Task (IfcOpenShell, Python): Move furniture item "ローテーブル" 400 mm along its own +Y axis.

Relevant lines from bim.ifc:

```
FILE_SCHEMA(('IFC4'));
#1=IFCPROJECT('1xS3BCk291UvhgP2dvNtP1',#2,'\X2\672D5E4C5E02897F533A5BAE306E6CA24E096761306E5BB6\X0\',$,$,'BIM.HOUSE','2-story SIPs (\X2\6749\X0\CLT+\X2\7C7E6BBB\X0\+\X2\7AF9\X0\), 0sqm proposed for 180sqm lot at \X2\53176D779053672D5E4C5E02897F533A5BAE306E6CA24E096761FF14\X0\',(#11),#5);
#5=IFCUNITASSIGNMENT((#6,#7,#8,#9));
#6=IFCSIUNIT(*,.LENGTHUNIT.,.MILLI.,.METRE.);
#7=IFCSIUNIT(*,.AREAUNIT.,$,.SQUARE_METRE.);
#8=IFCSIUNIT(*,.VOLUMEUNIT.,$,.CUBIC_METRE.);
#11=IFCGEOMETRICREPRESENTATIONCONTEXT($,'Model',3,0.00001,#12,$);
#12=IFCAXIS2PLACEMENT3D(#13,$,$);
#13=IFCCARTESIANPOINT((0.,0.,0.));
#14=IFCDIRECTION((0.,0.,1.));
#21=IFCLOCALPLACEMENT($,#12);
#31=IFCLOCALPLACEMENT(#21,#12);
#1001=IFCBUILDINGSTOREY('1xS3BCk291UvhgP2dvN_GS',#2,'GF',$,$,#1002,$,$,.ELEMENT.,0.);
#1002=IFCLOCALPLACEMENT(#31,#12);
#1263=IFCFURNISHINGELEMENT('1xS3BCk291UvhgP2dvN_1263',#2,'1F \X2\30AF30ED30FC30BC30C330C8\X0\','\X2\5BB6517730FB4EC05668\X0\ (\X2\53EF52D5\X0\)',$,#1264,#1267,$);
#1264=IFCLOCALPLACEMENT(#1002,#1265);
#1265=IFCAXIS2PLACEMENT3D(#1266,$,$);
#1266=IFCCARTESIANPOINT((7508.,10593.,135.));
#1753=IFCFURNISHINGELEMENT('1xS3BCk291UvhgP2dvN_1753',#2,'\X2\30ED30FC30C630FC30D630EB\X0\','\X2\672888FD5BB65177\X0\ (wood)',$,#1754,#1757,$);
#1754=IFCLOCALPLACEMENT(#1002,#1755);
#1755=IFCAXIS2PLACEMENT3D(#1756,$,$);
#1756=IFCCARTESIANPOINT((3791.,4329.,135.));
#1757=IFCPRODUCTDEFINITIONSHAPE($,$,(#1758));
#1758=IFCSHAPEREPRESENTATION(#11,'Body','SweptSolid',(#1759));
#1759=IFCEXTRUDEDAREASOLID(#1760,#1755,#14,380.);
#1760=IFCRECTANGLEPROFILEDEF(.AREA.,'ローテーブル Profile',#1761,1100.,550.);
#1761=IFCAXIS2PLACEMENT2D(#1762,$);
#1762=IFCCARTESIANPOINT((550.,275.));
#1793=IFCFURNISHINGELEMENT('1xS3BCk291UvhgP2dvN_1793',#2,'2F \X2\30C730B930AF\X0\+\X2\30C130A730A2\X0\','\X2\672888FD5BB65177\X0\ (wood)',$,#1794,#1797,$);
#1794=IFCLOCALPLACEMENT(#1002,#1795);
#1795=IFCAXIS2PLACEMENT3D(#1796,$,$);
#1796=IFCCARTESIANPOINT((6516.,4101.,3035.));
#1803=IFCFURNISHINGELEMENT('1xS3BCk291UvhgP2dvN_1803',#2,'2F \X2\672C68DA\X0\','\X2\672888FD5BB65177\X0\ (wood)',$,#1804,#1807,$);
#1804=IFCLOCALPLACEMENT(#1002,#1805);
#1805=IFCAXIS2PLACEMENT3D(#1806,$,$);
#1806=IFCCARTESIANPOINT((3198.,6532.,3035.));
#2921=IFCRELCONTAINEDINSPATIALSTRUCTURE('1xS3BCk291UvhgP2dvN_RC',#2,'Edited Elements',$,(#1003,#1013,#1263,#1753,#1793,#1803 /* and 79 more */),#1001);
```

```python
import ifcopenshell
import ifcopenshell.api.geometry
import ifcopenshell.util.placement
import ifcopenshell.util.unit

model = ifcopenshell.open("bim.ifc")
unit_scale = ifcopenshell.util.unit.calculate_unit_scale(model)

item = model.by_id(1753)
matrix = ifcopenshell.util.placement.get_local_placement(item.ObjectPlacement)
matrix[:3, 3] += matrix[:3, 1] * 0.4 / unit_scale
ifcopenshell.api.geometry.edit_object_placement(model, product=item, matrix=matrix, is_si=False)

print(ifcopenshell.util.placement.get_local_placement(item.ObjectPlacement).round(3) + 0.0)

model.write("bim_edited.ifc")
```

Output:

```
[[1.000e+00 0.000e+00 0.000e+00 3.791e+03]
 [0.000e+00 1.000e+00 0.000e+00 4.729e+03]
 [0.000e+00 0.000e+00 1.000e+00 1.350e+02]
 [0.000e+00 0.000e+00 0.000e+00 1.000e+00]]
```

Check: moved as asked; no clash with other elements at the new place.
